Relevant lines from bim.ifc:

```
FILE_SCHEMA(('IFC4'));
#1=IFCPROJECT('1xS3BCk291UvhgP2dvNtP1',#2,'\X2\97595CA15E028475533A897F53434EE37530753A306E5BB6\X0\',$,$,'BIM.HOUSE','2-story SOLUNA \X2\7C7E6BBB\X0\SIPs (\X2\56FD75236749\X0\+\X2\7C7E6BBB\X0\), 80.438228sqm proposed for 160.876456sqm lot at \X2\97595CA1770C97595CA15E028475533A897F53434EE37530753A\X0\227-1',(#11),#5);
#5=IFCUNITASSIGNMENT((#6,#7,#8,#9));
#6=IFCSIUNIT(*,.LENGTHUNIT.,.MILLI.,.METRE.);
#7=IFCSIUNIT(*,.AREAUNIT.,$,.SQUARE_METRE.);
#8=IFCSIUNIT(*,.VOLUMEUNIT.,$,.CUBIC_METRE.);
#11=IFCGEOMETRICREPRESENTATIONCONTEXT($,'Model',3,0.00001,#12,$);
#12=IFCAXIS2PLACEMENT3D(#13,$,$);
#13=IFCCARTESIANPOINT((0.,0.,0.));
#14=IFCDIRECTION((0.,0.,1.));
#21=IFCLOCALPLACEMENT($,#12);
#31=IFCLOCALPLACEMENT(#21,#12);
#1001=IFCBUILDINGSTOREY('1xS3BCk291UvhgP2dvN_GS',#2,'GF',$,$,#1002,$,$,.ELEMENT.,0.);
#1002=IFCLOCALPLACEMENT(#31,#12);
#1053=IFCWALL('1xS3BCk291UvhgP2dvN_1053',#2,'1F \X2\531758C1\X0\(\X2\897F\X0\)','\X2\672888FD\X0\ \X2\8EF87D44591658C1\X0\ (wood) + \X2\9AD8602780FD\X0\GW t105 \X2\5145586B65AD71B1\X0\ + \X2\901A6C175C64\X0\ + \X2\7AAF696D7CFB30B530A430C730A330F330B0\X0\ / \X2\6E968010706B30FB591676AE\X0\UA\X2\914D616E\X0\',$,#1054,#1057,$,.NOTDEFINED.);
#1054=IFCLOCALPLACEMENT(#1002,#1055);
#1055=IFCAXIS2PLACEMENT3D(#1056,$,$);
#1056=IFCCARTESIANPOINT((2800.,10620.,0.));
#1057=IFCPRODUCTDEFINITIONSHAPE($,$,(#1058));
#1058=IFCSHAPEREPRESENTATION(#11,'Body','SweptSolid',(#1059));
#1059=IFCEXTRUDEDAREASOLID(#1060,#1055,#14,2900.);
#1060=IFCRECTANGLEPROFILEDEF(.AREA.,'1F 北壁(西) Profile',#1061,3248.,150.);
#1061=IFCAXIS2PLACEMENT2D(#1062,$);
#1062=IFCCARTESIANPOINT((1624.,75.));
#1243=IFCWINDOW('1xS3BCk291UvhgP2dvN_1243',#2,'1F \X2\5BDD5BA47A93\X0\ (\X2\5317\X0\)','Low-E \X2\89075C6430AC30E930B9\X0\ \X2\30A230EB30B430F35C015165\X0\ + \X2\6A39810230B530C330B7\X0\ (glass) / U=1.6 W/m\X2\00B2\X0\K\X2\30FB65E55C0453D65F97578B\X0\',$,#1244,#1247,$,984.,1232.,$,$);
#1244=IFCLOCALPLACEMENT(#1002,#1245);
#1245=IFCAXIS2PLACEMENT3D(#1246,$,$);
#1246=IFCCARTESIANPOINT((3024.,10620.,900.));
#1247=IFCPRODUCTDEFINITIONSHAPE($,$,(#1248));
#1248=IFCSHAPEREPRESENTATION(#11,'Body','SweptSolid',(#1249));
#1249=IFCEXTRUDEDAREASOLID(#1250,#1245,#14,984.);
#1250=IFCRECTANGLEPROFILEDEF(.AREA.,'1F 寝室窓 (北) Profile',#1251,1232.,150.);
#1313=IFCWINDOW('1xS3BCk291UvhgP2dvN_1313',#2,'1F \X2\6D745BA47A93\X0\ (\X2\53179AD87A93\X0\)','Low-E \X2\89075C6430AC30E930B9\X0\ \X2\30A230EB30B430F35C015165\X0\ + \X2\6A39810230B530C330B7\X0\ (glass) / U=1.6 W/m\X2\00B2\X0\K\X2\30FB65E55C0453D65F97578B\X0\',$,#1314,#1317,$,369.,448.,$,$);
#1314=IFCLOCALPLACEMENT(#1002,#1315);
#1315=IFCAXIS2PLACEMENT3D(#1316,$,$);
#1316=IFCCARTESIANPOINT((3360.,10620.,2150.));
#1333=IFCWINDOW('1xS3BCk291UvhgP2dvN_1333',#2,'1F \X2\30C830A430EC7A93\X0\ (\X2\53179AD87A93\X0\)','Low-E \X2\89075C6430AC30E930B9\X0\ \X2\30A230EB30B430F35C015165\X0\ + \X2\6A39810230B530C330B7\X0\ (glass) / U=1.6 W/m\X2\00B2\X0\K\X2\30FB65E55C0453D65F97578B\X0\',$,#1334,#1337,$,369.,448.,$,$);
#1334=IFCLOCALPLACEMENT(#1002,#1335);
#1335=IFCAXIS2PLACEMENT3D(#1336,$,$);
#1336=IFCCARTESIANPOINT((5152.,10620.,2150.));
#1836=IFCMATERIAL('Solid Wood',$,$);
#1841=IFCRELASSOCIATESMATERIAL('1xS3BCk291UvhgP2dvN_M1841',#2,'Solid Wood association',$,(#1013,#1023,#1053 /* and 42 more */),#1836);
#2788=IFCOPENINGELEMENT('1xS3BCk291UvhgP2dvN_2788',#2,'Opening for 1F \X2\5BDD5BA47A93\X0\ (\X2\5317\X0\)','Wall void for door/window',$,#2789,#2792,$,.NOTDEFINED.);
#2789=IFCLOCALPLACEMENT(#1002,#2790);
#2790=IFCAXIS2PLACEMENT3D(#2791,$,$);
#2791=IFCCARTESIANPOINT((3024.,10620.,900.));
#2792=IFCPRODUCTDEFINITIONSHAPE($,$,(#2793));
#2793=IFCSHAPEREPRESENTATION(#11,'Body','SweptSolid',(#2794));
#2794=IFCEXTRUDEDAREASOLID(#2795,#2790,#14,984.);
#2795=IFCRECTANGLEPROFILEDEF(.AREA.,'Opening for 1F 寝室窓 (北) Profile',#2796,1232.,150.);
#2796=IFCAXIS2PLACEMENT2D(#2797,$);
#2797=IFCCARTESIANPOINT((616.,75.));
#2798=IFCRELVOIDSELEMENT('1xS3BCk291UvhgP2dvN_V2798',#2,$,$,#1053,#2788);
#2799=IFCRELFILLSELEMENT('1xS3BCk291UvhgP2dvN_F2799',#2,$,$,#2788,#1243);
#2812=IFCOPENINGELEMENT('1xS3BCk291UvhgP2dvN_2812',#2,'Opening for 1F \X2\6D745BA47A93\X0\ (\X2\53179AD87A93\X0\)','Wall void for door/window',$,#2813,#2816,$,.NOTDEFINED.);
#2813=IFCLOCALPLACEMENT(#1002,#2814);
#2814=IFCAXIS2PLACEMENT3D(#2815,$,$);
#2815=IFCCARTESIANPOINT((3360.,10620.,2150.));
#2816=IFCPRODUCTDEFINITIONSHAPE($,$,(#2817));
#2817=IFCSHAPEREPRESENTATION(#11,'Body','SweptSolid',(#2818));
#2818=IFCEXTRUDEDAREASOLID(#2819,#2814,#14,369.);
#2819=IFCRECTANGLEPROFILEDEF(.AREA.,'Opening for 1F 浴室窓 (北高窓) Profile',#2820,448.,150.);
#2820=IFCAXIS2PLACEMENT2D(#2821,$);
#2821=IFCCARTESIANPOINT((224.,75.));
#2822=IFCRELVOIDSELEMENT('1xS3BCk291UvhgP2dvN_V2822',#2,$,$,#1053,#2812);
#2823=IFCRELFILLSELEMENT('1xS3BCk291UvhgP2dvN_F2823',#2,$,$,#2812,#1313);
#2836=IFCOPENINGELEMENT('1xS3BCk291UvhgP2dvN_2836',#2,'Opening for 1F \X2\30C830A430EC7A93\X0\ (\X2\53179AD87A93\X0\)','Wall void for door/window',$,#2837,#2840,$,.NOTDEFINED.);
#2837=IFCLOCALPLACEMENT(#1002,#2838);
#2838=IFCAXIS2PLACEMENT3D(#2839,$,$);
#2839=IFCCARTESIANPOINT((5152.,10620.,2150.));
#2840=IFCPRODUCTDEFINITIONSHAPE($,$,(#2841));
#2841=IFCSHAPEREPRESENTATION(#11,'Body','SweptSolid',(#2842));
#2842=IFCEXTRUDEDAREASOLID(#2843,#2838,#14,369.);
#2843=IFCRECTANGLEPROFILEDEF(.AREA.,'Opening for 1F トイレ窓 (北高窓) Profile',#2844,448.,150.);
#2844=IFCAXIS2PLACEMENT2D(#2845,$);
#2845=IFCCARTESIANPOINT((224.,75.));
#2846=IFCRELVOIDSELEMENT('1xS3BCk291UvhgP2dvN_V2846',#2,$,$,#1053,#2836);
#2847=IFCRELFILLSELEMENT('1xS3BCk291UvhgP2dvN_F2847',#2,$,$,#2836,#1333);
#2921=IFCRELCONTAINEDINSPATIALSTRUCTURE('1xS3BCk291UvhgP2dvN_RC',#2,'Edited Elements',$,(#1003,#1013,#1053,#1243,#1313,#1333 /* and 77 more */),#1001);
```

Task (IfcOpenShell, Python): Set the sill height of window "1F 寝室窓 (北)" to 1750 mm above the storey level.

```python
import numpy as np
import ifcopenshell
import ifcopenshell.api.geometry
import ifcopenshell.geom
import ifcopenshell.util.element
import ifcopenshell.util.placement
import ifcopenshell.util.shape
import ifcopenshell.util.unit

model = ifcopenshell.open("bim.ifc")
unit_scale = ifcopenshell.util.unit.calculate_unit_scale(model)

window = model.by_guid("1xS3BCk291UvhgP2dvN_1243")
opening = window.FillsVoids[0].RelatingOpeningElement
storey = ifcopenshell.util.element.get_container(window, ifc_class="IfcBuildingStorey")
level = ifcopenshell.util.placement.get_local_placement(storey.ObjectPlacement)[2, 3]

# The opening's origin need not be at the sill, so measure its lowest point.
shape = ifcopenshell.geom.create_shape(ifcopenshell.geom.settings(), opening)
bottom = ifcopenshell.util.shape.get_shape_bottom_elevation(shape, shape.geometry) / unit_scale
dz = level + 1750.0 - bottom

shift = np.array([0.0, 0.0, dz])
# The window is not placed relative to its opening, so move both.
for product in (opening, window):
    matrix = ifcopenshell.util.placement.get_local_placement(product.ObjectPlacement)
    matrix[:3, 3] += shift
    ifcopenshell.api.geometry.edit_object_placement(model, product=product, matrix=matrix, is_si=False)

print(f"moved by {dz * unit_scale:+.3f} m")

model.write("bim-out.ifc")
```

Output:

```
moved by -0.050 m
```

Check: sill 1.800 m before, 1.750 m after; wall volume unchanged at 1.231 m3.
